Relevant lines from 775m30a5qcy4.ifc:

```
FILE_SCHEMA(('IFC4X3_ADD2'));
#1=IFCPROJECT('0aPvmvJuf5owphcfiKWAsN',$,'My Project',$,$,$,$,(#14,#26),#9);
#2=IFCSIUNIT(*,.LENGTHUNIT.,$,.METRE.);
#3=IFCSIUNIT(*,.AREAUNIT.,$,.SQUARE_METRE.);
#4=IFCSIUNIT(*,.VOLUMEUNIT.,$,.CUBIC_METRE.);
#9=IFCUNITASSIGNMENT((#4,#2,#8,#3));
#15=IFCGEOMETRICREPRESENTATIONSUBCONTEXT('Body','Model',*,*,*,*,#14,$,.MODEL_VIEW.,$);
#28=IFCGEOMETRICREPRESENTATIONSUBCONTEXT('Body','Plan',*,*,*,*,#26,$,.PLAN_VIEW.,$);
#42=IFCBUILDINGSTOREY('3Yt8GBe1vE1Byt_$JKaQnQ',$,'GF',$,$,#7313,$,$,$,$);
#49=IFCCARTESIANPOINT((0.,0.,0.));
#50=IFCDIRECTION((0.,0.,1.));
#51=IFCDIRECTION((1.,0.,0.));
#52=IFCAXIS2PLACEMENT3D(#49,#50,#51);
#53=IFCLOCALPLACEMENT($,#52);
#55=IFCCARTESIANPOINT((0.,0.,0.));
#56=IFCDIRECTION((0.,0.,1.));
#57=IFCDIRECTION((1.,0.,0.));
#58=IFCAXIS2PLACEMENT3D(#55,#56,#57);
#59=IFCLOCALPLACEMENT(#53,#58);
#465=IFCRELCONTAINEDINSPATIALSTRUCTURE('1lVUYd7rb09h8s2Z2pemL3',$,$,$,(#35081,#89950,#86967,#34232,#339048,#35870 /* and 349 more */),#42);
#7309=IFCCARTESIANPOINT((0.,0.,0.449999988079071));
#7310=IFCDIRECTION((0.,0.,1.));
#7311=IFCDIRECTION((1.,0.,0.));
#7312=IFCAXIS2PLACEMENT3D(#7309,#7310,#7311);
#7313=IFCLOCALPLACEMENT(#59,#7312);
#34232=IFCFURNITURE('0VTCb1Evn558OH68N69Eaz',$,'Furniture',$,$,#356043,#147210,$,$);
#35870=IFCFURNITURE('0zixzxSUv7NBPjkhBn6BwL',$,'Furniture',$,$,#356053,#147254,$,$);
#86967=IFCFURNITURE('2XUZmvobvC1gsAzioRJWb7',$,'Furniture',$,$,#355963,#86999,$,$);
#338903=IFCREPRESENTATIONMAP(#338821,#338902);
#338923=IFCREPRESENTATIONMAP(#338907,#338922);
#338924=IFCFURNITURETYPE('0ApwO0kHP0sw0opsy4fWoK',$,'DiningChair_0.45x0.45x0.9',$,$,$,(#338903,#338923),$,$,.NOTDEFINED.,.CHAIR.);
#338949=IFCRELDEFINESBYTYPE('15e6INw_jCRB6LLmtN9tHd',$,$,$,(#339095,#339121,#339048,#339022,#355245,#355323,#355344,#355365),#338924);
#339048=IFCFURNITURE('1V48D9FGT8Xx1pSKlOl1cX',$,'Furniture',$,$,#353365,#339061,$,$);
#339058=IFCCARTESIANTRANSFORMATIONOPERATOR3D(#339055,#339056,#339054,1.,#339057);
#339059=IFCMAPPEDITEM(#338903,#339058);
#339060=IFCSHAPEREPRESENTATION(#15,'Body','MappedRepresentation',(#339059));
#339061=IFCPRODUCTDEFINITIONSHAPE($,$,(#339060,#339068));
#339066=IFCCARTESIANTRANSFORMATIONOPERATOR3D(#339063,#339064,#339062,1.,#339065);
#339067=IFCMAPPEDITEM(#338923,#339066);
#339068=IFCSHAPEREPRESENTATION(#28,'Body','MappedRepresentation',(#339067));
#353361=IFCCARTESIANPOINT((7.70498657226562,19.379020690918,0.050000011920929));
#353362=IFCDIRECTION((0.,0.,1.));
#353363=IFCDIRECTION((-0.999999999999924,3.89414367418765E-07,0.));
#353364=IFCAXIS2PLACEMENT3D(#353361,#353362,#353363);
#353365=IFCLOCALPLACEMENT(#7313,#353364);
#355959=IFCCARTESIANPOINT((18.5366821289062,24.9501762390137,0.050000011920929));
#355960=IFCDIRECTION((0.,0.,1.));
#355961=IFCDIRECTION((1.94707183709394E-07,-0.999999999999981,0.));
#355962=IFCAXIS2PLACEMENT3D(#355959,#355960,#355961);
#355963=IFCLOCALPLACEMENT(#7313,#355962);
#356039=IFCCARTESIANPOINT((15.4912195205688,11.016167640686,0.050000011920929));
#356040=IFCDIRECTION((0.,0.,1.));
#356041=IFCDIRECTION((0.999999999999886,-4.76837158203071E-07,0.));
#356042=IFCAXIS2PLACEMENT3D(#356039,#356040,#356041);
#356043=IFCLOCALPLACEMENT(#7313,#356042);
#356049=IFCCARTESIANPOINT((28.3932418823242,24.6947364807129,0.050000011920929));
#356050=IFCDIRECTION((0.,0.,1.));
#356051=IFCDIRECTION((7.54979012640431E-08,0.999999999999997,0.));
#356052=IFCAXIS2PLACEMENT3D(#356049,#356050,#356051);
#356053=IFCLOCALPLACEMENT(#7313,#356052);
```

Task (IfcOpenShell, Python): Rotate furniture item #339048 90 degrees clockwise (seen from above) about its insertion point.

```python
import ifcopenshell
import ifcopenshell.api.geometry
import ifcopenshell.util.placement

model = ifcopenshell.open("775m30a5qcy4.ifc")

item = model.by_guid("1V48D9FGT8Xx1pSKlOl1cX")
matrix = ifcopenshell.util.placement.get_local_placement(item.ObjectPlacement)
matrix = matrix @ ifcopenshell.util.placement.rotation(-90, "Z")
ifcopenshell.api.geometry.edit_object_placement(model, product=item, matrix=matrix, is_si=False)

print(ifcopenshell.util.placement.get_local_placement(item.ObjectPlacement).round(3) + 0.0)

model.write("775m30a5qcy4_v2.ifc")
```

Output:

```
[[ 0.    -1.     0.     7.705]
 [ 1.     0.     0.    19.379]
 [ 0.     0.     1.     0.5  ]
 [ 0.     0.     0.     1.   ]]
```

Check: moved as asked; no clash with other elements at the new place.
